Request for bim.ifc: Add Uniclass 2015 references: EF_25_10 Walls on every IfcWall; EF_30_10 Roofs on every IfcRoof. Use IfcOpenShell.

First a look at what the model holds.

```python
import ifcopenshell

model = ifcopenshell.open("bim.ifc")
print(model.schema)
print("classifications:", [c.Name for c in model.by_type("IfcClassification")])
for ifc_class in ("IfcDoor", "IfcRoof", "IfcStair", "IfcWall", "IfcWindow"):
    print(ifc_class, len(model.by_type(ifc_class)))
```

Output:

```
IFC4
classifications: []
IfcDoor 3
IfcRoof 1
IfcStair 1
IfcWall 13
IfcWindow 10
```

```python
import ifcopenshell
import ifcopenshell.api.classification

model = ifcopenshell.open("bim.ifc")

system = ifcopenshell.api.classification.add_classification(model, classification="Uniclass 2015")

codes = {
    "IfcWall": ("EF_25_10", "Walls"),
    "IfcRoof": ("EF_30_10", "Roofs"),
}
for ifc_class, (code, name) in codes.items():
    products = model.by_type(ifc_class)
    ifcopenshell.api.classification.add_reference(
        model, products=products, classification=system, identification=code, name=name
    )
    print(code, len(products))

model.write("bim_rev.ifc")
```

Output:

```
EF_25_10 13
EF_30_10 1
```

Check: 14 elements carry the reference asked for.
